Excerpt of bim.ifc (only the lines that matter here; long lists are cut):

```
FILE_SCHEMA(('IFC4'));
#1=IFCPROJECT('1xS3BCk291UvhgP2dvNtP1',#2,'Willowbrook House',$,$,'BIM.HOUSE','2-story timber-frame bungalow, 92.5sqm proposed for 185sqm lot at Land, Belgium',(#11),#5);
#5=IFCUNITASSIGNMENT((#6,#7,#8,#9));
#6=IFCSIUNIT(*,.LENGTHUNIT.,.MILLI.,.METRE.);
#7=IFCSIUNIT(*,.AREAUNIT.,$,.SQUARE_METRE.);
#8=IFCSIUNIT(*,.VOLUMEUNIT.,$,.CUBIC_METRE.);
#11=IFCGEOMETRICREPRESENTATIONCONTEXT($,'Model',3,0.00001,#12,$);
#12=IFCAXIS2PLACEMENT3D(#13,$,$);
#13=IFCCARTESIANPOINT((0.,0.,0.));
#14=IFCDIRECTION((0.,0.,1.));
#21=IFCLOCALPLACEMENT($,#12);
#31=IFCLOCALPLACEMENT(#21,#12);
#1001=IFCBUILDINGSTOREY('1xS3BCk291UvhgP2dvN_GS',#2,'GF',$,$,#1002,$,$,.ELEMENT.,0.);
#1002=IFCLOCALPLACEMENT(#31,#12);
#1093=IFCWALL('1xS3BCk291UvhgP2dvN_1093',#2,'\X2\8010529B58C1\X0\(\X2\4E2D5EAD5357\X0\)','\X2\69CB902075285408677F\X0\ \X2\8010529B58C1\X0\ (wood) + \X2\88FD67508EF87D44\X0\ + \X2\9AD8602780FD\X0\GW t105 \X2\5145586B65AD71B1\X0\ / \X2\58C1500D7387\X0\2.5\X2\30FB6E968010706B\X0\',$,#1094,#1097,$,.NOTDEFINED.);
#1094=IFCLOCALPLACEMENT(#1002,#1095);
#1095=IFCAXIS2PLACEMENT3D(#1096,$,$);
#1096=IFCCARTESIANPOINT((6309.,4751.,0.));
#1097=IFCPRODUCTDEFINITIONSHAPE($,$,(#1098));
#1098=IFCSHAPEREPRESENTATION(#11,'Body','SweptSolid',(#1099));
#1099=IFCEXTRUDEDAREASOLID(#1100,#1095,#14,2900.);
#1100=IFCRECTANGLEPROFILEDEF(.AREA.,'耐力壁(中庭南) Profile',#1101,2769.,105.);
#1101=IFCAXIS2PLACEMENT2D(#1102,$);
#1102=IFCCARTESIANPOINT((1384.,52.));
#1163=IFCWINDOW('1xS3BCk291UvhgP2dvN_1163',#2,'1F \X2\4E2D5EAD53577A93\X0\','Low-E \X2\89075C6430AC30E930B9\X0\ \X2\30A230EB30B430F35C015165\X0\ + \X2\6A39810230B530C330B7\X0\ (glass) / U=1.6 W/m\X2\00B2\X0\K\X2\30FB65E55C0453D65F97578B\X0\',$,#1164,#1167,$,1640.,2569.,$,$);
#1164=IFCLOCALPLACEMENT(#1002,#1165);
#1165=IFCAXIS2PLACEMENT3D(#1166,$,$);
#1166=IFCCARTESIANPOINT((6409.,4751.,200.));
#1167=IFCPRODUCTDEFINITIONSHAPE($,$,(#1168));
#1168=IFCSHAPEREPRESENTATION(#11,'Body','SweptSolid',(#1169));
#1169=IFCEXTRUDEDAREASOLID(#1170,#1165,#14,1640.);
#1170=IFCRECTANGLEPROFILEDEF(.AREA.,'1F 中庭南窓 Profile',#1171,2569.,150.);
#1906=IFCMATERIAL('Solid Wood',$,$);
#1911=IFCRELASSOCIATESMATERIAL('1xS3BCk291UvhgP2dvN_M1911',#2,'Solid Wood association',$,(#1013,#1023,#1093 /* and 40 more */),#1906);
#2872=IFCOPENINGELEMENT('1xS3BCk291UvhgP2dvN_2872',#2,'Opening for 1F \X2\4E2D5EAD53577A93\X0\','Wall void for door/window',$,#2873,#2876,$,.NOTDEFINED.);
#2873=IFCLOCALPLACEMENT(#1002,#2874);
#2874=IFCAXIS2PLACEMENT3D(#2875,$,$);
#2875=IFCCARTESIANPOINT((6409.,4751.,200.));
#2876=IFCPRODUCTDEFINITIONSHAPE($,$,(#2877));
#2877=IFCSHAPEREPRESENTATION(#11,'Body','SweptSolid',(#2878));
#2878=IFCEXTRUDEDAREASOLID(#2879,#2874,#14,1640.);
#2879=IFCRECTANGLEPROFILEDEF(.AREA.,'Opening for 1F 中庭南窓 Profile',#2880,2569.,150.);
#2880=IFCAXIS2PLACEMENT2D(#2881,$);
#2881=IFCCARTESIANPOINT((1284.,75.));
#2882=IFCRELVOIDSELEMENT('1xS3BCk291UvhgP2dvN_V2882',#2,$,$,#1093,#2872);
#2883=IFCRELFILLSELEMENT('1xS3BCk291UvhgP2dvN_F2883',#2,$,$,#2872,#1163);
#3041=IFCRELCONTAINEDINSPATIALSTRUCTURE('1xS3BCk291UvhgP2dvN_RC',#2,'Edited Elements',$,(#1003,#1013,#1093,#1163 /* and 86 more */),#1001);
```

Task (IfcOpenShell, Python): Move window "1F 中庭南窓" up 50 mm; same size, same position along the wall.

```python
import numpy as np
import ifcopenshell
import ifcopenshell.api.geometry
import ifcopenshell.util.placement
import ifcopenshell.util.unit

model = ifcopenshell.open("bim.ifc")
unit_scale = ifcopenshell.util.unit.calculate_unit_scale(model)

window = model.by_guid("1xS3BCk291UvhgP2dvN_1163")
opening = window.FillsVoids[0].RelatingOpeningElement
dz = 0.05 / unit_scale

shift = np.array([0.0, 0.0, dz])
# The window is not placed relative to its opening, so move both.
for product in (opening, window):
    matrix = ifcopenshell.util.placement.get_local_placement(product.ObjectPlacement)
    matrix[:3, 3] += shift
    ifcopenshell.api.geometry.edit_object_placement(model, product=product, matrix=matrix, is_si=False)

print(f"moved by {dz * unit_scale:+.3f} m")

model.write("bim_v2.ifc")
```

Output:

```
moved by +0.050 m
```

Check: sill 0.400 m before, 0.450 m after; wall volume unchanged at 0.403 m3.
